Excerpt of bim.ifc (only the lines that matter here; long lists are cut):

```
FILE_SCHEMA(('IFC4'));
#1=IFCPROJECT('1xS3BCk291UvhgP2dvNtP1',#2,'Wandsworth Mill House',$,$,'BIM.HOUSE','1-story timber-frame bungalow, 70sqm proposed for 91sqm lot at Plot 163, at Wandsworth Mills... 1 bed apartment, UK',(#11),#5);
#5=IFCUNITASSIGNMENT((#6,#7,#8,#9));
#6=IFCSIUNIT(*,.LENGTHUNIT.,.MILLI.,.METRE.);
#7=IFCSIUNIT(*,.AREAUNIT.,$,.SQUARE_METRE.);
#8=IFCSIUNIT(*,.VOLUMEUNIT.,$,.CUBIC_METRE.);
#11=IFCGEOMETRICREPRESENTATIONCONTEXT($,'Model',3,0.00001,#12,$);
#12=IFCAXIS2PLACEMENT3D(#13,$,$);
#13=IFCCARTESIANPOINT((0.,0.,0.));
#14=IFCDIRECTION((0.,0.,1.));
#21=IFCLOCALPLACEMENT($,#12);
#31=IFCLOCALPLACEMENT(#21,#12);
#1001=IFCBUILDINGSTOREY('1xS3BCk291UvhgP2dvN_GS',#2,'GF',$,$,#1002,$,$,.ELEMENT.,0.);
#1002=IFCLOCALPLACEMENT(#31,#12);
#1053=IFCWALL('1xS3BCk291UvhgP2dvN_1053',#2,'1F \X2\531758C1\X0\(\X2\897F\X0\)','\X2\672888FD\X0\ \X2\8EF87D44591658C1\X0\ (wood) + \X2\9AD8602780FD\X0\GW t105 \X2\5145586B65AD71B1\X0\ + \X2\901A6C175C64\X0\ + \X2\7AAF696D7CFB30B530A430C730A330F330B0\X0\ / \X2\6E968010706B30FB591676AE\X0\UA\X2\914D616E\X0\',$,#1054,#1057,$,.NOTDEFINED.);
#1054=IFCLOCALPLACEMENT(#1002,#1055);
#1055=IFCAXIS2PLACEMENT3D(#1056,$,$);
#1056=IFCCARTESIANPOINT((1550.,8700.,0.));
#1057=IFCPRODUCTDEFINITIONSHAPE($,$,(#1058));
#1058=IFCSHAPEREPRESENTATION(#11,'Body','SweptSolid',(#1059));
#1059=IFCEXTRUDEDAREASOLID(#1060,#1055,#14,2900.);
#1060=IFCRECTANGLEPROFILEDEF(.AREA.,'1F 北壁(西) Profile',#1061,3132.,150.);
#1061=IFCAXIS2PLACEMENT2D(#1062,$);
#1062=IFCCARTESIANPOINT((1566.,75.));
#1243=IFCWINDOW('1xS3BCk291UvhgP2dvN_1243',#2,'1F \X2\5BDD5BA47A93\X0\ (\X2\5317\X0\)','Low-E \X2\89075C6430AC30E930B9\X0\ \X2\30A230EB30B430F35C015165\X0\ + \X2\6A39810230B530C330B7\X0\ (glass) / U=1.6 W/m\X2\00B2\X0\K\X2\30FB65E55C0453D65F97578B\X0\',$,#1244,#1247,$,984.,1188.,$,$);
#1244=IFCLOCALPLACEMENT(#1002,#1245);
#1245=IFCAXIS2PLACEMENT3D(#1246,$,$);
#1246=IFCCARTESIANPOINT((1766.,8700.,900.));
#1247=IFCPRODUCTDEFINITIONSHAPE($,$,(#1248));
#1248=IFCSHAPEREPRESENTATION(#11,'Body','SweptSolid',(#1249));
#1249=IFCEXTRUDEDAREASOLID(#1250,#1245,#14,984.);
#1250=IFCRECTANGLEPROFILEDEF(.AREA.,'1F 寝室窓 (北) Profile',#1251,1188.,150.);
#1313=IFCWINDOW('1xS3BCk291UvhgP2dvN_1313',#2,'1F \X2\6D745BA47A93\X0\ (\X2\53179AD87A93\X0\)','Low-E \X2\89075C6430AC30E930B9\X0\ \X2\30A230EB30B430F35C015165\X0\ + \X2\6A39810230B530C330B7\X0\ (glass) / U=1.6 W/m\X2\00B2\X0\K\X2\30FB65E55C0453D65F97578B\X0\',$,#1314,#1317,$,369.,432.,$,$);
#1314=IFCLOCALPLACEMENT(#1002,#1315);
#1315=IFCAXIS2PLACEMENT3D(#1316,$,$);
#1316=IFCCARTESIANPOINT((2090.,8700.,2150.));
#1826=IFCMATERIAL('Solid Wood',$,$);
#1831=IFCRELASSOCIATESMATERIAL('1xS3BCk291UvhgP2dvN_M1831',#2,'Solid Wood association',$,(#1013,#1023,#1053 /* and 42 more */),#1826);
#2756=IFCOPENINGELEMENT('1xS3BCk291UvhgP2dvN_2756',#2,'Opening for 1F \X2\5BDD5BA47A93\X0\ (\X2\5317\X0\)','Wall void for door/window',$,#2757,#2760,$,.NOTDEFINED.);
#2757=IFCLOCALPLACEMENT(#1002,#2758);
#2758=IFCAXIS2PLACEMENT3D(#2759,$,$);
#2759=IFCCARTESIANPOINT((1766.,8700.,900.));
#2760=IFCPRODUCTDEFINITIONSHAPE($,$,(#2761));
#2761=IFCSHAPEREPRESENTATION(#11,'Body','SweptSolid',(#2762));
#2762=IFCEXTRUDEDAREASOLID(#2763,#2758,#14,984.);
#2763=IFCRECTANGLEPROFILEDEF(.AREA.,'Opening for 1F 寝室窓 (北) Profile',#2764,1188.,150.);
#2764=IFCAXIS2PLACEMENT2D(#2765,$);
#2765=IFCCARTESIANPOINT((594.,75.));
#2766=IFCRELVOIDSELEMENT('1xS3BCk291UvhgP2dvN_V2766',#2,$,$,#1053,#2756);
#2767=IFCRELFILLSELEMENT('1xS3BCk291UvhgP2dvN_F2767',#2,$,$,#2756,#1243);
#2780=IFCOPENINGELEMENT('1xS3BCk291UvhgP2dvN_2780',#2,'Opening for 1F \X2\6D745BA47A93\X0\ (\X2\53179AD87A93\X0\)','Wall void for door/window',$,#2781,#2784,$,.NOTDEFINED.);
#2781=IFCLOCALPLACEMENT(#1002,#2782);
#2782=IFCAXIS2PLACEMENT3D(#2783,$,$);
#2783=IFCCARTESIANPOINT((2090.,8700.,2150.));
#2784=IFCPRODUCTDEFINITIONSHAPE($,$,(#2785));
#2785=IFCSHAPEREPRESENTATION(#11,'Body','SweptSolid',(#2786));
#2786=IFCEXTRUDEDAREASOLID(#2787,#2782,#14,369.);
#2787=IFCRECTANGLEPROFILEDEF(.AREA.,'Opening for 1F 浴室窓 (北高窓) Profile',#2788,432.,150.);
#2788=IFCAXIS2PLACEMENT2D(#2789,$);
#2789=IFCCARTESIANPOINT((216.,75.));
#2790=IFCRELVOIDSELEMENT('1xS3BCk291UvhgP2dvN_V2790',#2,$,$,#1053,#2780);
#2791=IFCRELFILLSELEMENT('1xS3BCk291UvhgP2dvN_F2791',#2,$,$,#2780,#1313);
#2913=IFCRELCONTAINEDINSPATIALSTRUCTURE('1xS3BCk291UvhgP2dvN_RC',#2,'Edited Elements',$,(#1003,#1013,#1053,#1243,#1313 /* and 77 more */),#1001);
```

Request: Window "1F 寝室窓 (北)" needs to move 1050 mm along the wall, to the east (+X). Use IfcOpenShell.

```python
import ifcopenshell
import ifcopenshell.api.geometry
import ifcopenshell.util.placement
import ifcopenshell.util.unit

model = ifcopenshell.open("bim.ifc")
unit_scale = ifcopenshell.util.unit.calculate_unit_scale(model)

window = model.by_guid("1xS3BCk291UvhgP2dvN_1243")
opening = window.FillsVoids[0].RelatingOpeningElement
wall = opening.VoidsElements[0].RelatingBuildingElement

wall_matrix = ifcopenshell.util.placement.get_local_placement(wall.ObjectPlacement)
shift = wall_matrix[:3, 0] * 1.05 / unit_scale
before = ifcopenshell.util.placement.get_local_placement(window.ObjectPlacement)[:3, 3].copy()

# The window is not placed relative to its opening, so move both.
for product in (opening, window):
    matrix = ifcopenshell.util.placement.get_local_placement(product.ObjectPlacement)
    matrix[:3, 3] += shift
    ifcopenshell.api.geometry.edit_object_placement(model, product=product, matrix=matrix, is_si=False)

after = ifcopenshell.util.placement.get_local_placement(window.ObjectPlacement)[:3, 3]
print("window moved by", (after - before).round(3) + 0.0)

model.write("bim_rev.ifc")
```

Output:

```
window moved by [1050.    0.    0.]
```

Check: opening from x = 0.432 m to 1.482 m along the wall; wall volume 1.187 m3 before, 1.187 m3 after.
